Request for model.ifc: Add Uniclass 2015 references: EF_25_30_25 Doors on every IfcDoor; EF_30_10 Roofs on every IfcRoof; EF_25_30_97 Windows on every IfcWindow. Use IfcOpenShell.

First a look at what the model holds.

```python
import ifcopenshell

model = ifcopenshell.open("model.ifc")
print(model.schema)
print("classifications:", [c.Name for c in model.by_type("IfcClassification")])
for ifc_class in ("IfcDoor", "IfcRoof", "IfcStair", "IfcWall", "IfcWindow"):
    print(ifc_class, len(model.by_type(ifc_class)))
```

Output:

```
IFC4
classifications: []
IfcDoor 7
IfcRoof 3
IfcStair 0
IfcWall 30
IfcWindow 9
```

```python
import ifcopenshell
import ifcopenshell.api.classification

model = ifcopenshell.open("model.ifc")

system = ifcopenshell.api.classification.add_classification(model, classification="Uniclass 2015")

codes = {
    "IfcDoor": ("EF_25_30_25", "Doors"),
    "IfcRoof": ("EF_30_10", "Roofs"),
    "IfcWindow": ("EF_25_30_97", "Windows"),
}
for ifc_class, (code, name) in codes.items():
    products = model.by_type(ifc_class)
    ifcopenshell.api.classification.add_reference(
        model, products=products, classification=system, identification=code, name=name
    )
    print(code, len(products))

model.write("model_updated.ifc")
```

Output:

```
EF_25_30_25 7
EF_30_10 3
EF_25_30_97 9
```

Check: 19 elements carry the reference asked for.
